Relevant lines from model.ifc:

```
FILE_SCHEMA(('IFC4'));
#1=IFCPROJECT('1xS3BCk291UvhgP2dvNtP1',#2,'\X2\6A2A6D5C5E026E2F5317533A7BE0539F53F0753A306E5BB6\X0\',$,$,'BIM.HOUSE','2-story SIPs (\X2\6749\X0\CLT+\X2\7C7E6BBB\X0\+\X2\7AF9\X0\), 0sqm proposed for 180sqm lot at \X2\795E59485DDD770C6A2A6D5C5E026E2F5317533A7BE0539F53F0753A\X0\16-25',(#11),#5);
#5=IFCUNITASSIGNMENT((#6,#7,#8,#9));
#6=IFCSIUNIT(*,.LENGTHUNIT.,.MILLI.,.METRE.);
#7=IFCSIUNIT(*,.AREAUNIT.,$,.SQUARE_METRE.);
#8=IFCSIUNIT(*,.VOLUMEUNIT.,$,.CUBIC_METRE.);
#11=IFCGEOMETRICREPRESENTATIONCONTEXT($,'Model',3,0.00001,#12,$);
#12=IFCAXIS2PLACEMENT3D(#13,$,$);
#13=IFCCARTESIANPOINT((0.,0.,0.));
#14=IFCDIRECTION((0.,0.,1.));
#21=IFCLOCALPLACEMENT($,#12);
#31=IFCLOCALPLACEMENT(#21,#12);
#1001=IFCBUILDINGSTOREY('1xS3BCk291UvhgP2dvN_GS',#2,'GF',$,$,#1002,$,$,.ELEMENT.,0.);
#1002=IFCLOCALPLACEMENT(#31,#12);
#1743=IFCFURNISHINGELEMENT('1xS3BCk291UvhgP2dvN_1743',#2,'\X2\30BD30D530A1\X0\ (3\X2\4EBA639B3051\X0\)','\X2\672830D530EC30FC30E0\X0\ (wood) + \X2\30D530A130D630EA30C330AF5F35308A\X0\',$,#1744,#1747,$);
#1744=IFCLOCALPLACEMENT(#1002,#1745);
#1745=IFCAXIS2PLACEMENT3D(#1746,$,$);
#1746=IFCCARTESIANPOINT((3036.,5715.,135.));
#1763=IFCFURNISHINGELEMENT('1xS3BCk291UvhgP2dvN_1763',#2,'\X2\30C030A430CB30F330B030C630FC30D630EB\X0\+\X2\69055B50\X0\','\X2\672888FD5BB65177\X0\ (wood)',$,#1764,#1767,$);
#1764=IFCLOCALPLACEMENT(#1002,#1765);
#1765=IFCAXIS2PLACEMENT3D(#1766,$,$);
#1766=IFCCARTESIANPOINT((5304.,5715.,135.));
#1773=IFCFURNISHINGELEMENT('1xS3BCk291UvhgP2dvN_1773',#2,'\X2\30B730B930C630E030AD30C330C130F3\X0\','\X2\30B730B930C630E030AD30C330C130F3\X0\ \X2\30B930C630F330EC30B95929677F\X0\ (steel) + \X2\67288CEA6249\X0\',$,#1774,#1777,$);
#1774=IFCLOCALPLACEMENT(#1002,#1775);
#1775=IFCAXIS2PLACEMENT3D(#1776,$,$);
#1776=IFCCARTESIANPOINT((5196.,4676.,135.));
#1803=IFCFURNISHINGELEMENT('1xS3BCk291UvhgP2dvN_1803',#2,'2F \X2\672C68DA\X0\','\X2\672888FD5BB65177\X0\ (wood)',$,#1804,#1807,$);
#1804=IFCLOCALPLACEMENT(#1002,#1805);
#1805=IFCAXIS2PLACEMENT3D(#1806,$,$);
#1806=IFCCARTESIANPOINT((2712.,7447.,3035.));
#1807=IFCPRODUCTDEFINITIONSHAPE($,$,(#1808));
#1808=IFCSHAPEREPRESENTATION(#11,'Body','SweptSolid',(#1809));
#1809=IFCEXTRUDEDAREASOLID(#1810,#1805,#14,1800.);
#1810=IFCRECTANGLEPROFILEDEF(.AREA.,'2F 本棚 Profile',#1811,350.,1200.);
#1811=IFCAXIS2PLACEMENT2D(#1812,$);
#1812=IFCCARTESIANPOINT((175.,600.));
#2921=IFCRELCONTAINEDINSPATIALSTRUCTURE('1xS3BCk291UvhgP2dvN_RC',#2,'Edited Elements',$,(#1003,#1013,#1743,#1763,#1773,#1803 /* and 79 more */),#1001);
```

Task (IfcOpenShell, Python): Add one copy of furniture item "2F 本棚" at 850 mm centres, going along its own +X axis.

```python
import ifcopenshell
import ifcopenshell.api.geometry
import ifcopenshell.api.root
import ifcopenshell.util.element
import ifcopenshell.util.placement

model = ifcopenshell.open("model.ifc")


def reuse_history(source, copy):
    """copy_class also copies each property set's owner history, people and application; keep the originals."""
    for rel in copy.IsDefinedBy:
        if rel.is_a("IfcRelDefinesByProperties") and (history := rel.RelatingPropertyDefinition.OwnerHistory):
            rel.RelatingPropertyDefinition.OwnerHistory = source.OwnerHistory
            ifcopenshell.util.element.remove_deep2(model, history)


source = model.by_guid("1xS3BCk291UvhgP2dvN_1803")
base = ifcopenshell.util.placement.get_local_placement(source.ObjectPlacement)
step = base[:3, 0] * 850.0

for i in range(1, 2):
    copy = ifcopenshell.api.root.copy_class(model, product=source)
    copy.Representation = ifcopenshell.util.element.copy_deep(
        model, source.Representation, exclude=["IfcGeometricRepresentationContext", "IfcRepresentationMap"]
    )
    reuse_history(source, copy)
    matrix = base.copy()
    matrix[:3, 3] += i * step
    print("added at", matrix[:3, 3].round(3) + 0.0)
    ifcopenshell.api.geometry.edit_object_placement(model, product=copy, matrix=matrix, is_si=False)

model.write("model-out.ifc")
```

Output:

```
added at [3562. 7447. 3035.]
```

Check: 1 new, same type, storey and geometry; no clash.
